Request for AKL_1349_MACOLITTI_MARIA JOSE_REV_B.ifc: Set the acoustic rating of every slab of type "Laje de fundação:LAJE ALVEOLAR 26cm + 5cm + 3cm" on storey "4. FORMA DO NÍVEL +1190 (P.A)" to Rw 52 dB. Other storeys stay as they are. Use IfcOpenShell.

First a look at what the model holds.

```python
import ifcopenshell
import ifcopenshell.util.element

model = ifcopenshell.open("AKL_1349_MACOLITTI_MARIA JOSE_REV_B.ifc")
print(model.schema)
storey = next(s for s in model.by_type("IfcBuildingStorey") if s.Name == "4. FORMA DO NÍVEL +1190 (P.A)")
slabs = [e for e in ifcopenshell.util.element.get_decomposition(storey) if e.is_a("IfcSlab")]
seen = {}
for e in slabs:
    element_type = ifcopenshell.util.element.get_type(e)
    key = (element_type.Name if element_type != e and element_type else None, ifcopenshell.util.element.get_pset(e, "Pset_SlabCommon", "AcousticRating"))
    seen[key] = seen.get(key, 0) + 1
for (name, value), count in sorted(seen.items(), key=str):
    print(count, "x", name, "|", value)
```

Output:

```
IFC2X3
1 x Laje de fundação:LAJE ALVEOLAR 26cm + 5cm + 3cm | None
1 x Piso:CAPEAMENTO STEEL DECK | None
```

```python
import ifcopenshell
import ifcopenshell.api.pset
import ifcopenshell.util.element

model = ifcopenshell.open("AKL_1349_MACOLITTI_MARIA JOSE_REV_B.ifc")

storey = next(s for s in model.by_type("IfcBuildingStorey") if s.Name == "4. FORMA DO NÍVEL +1190 (P.A)")
slabs = [e for e in ifcopenshell.util.element.get_decomposition(storey) if e.is_a("IfcSlab")]

count = 0
for e in slabs:
    element_type = ifcopenshell.util.element.get_type(e)
    if element_type in (None, e) or element_type.Name != "Laje de fundação:LAJE ALVEOLAR 26cm + 5cm + 3cm":
        continue
    # add_pset returns the element's existing set when there is one.
    pset = ifcopenshell.api.pset.add_pset(model, product=e, name="Pset_SlabCommon")
    ifcopenshell.api.pset.edit_pset(model, pset=pset, properties={"AcousticRating": "Rw 52 dB"})
    count += 1

print(count, "slabs updated")

model.write("AKL_1349_MACOLITTI_MARIA JOSE_REV_B-out.ifc")
```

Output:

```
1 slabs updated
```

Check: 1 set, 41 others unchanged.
